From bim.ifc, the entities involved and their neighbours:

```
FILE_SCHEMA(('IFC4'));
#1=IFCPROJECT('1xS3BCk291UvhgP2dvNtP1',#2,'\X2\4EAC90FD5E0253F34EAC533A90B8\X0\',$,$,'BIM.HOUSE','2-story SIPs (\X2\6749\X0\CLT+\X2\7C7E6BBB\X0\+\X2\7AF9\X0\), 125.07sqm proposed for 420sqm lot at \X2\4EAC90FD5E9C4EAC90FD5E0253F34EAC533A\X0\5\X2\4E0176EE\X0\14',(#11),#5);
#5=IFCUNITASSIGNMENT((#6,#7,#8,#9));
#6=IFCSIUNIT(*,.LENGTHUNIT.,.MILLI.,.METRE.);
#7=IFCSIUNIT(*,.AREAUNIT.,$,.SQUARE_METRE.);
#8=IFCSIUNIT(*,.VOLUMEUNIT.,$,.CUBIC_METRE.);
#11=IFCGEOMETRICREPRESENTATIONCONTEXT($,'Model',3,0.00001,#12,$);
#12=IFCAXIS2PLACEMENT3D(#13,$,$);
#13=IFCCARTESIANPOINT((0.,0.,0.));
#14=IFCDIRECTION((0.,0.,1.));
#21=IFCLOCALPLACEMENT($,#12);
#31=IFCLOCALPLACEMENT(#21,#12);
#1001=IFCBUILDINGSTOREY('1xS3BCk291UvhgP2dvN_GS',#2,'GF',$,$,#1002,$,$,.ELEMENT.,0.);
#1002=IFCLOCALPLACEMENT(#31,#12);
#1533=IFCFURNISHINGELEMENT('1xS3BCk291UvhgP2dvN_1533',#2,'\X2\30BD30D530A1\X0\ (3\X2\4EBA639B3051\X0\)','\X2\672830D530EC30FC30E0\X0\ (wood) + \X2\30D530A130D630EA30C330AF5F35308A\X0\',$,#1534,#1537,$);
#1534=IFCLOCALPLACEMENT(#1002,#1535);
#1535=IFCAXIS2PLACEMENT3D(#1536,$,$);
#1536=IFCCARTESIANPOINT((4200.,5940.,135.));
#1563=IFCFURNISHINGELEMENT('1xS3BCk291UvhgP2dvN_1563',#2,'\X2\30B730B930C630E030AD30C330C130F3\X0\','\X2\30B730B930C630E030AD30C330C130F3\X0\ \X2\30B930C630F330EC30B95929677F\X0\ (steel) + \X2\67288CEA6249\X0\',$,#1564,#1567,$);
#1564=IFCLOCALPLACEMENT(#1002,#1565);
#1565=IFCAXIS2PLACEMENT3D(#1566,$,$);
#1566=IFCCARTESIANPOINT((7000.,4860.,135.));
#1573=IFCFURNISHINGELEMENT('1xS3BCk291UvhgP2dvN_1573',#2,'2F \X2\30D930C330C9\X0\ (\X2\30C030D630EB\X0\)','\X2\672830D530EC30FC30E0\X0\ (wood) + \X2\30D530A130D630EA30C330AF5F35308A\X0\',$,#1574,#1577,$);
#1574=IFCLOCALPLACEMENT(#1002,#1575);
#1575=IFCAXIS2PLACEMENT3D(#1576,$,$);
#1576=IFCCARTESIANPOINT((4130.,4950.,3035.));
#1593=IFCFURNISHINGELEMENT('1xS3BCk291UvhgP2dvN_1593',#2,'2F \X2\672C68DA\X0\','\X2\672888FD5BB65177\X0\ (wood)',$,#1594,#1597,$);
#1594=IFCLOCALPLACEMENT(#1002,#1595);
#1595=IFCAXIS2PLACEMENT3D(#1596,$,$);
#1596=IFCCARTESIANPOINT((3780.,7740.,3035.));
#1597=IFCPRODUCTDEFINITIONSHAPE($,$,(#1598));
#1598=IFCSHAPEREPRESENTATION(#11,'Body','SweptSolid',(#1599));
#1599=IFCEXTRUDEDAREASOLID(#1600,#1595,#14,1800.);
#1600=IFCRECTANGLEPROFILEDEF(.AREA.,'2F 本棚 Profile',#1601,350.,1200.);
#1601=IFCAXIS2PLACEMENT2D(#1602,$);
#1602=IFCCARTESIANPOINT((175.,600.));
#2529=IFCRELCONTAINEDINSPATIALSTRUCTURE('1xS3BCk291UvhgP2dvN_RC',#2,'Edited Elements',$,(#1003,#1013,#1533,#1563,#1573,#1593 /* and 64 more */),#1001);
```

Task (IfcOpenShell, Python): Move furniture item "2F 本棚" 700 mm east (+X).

```python
import ifcopenshell
import ifcopenshell.api.geometry
import ifcopenshell.util.placement
import ifcopenshell.util.unit

model = ifcopenshell.open("bim.ifc")
unit_scale = ifcopenshell.util.unit.calculate_unit_scale(model)

item = model.by_guid("1xS3BCk291UvhgP2dvN_1593")
matrix = ifcopenshell.util.placement.get_local_placement(item.ObjectPlacement)
matrix[0, 3] += 0.7 / unit_scale
ifcopenshell.api.geometry.edit_object_placement(model, product=item, matrix=matrix, is_si=False)

print(ifcopenshell.util.placement.get_local_placement(item.ObjectPlacement).round(3) + 0.0)

model.write("bim_edited.ifc")
```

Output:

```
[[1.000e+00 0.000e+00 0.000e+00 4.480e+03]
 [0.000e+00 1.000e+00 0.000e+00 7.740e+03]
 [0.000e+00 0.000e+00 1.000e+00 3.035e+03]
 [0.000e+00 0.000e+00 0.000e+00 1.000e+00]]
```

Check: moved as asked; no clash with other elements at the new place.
